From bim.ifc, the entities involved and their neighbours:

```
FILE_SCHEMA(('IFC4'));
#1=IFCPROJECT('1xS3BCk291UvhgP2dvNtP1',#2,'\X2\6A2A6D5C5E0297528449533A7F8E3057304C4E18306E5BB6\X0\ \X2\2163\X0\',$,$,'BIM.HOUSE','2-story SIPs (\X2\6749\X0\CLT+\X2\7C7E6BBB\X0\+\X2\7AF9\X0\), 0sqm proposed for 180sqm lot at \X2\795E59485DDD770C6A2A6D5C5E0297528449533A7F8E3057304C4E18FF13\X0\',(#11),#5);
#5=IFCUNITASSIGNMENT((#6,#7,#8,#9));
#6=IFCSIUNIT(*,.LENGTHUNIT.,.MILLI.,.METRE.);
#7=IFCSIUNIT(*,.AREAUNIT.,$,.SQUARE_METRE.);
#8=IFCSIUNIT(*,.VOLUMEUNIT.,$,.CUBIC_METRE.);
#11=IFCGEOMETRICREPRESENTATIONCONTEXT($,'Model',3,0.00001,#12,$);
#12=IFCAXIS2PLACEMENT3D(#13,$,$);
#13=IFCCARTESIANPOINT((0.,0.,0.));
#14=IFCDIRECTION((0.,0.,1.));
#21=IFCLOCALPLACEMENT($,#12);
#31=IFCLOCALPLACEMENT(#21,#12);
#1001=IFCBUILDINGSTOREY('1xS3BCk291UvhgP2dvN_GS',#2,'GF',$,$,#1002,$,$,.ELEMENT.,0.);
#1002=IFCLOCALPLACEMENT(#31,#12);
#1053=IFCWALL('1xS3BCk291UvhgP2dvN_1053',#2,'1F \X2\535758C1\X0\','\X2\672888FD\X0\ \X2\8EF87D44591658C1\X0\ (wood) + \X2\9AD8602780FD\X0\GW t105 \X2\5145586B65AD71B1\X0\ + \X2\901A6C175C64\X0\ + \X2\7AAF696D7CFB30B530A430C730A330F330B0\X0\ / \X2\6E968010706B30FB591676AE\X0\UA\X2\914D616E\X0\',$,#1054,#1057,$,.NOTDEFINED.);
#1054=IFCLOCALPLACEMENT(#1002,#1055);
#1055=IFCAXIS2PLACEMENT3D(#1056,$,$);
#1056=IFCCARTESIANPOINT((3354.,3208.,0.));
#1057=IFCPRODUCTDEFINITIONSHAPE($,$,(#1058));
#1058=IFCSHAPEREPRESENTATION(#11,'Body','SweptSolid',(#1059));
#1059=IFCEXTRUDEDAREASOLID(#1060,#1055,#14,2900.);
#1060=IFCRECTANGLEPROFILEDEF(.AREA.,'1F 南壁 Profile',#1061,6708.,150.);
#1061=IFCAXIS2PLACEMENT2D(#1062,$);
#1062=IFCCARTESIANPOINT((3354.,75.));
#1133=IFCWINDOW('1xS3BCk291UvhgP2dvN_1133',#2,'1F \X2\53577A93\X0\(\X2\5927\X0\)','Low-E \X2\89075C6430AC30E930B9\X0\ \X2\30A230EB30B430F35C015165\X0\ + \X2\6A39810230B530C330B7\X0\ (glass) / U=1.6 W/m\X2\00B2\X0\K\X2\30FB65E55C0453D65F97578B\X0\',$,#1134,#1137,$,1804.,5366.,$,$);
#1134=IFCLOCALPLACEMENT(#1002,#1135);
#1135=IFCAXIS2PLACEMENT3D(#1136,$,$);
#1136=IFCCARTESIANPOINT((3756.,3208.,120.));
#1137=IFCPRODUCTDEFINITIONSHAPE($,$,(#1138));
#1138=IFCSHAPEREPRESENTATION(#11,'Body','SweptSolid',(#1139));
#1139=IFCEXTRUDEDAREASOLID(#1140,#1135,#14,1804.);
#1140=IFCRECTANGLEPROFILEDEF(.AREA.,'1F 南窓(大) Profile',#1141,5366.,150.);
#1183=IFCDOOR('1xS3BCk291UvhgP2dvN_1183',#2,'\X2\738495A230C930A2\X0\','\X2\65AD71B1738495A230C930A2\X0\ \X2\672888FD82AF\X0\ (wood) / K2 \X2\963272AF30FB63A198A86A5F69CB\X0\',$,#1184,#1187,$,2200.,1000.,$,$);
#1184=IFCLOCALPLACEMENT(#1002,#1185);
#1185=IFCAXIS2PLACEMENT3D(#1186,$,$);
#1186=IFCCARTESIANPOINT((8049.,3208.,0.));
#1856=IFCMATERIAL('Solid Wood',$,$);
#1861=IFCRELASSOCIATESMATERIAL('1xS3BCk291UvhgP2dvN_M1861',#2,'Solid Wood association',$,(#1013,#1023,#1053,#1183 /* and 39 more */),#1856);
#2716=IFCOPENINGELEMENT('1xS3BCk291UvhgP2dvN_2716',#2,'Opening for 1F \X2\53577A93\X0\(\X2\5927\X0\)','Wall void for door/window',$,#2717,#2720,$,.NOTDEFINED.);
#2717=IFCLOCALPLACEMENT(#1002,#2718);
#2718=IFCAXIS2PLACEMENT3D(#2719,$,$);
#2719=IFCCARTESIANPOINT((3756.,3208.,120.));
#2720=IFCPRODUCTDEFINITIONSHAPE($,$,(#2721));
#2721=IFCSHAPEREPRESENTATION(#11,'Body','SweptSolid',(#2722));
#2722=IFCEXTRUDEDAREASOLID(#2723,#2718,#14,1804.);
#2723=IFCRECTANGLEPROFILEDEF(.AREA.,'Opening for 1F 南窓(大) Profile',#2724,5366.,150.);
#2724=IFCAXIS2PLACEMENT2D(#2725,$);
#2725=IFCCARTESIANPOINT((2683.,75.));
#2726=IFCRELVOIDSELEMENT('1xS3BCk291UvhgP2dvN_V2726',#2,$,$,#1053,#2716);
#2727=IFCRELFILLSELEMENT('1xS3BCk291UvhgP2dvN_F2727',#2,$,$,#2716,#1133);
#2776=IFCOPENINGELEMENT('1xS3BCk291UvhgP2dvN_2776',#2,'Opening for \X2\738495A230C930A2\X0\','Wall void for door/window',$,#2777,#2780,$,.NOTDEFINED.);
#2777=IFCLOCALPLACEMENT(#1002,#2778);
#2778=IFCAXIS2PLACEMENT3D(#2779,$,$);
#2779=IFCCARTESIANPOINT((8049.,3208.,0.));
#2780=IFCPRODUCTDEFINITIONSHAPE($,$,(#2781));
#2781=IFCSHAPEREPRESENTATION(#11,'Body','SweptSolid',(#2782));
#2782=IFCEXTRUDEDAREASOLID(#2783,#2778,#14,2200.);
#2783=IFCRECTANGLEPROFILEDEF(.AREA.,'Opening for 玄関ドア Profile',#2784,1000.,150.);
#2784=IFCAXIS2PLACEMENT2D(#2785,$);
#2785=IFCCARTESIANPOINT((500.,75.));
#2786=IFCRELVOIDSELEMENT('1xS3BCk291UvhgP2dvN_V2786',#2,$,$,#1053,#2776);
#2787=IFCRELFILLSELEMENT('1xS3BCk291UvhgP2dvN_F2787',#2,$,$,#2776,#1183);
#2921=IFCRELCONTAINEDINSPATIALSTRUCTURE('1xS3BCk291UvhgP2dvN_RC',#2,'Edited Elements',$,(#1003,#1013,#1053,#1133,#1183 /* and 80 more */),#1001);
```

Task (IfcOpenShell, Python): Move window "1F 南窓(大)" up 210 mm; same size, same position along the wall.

```python
import numpy as np
import ifcopenshell
import ifcopenshell.api.geometry
import ifcopenshell.util.placement
import ifcopenshell.util.unit

model = ifcopenshell.open("bim.ifc")
unit_scale = ifcopenshell.util.unit.calculate_unit_scale(model)

window = model.by_id(1133)
opening = window.FillsVoids[0].RelatingOpeningElement
dz = 0.21 / unit_scale

shift = np.array([0.0, 0.0, dz])
# The window is not placed relative to its opening, so move both.
for product in (opening, window):
    matrix = ifcopenshell.util.placement.get_local_placement(product.ObjectPlacement)
    matrix[:3, 3] += shift
    ifcopenshell.api.geometry.edit_object_placement(model, product=product, matrix=matrix, is_si=False)

print(f"moved by {dz * unit_scale:+.3f} m")

model.write("bim_rev.ifc")
```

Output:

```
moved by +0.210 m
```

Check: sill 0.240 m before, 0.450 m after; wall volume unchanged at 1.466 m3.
